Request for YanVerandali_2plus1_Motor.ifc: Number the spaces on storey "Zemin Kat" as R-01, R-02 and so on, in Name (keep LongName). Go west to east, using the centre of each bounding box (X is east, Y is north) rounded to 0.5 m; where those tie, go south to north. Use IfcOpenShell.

First a look at what the model holds.

```python
import ifcopenshell
import ifcopenshell.util.element
import ifcopenshell.util.placement

model = ifcopenshell.open("YanVerandali_2plus1_Motor.ifc")
print(model.schema)
storey = next(s for s in model.by_type("IfcBuildingStorey") if s.Name == "Zemin Kat")
spaces = [e for e in ifcopenshell.util.element.get_decomposition(storey) if e.is_a("IfcSpace")]
for e in sorted(spaces, key=lambda e: e.id()):
    origin = ifcopenshell.util.placement.get_local_placement(e.ObjectPlacement)[:3, 3]
    print(e.id(), e.Name, e.LongName, origin.round(2) + 0.0, sep=" | ")
```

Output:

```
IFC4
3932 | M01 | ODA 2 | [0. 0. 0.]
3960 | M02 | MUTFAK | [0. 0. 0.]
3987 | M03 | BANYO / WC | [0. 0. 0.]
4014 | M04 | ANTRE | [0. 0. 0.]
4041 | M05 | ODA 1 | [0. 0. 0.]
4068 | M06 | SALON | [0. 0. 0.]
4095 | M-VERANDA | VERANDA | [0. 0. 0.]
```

```python
import ifcopenshell
import ifcopenshell.geom
import ifcopenshell.util.element
import ifcopenshell.util.shape

model = ifcopenshell.open("YanVerandali_2plus1_Motor.ifc")
settings = ifcopenshell.geom.settings()
settings.set("use-world-coords", True)


def centre(element):
    shape = ifcopenshell.geom.create_shape(settings, element)
    return ifcopenshell.util.shape.get_bbox_centroid(shape.geometry)


storey = next(s for s in model.by_type("IfcBuildingStorey") if s.Name == "Zemin Kat")
spaces = [e for e in ifcopenshell.util.element.get_decomposition(storey) if e.is_a("IfcSpace")]

# Insertion points can sit at a corner or the storey origin, so sort by the geometry (in metres).
centres = {e: centre(e) for e in spaces}
spaces.sort(key=lambda e: (round(centres[e][0] / 0.5), centres[e][1]))

for i, e in enumerate(spaces, start=1):
    number = f"R-{i:02d}"
    e.Name = number
    print(e.id(), number)

model.write("YanVerandali_2plus1_Motor-out.ifc")
```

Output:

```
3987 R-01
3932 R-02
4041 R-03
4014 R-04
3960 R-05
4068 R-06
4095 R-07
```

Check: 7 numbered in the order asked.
